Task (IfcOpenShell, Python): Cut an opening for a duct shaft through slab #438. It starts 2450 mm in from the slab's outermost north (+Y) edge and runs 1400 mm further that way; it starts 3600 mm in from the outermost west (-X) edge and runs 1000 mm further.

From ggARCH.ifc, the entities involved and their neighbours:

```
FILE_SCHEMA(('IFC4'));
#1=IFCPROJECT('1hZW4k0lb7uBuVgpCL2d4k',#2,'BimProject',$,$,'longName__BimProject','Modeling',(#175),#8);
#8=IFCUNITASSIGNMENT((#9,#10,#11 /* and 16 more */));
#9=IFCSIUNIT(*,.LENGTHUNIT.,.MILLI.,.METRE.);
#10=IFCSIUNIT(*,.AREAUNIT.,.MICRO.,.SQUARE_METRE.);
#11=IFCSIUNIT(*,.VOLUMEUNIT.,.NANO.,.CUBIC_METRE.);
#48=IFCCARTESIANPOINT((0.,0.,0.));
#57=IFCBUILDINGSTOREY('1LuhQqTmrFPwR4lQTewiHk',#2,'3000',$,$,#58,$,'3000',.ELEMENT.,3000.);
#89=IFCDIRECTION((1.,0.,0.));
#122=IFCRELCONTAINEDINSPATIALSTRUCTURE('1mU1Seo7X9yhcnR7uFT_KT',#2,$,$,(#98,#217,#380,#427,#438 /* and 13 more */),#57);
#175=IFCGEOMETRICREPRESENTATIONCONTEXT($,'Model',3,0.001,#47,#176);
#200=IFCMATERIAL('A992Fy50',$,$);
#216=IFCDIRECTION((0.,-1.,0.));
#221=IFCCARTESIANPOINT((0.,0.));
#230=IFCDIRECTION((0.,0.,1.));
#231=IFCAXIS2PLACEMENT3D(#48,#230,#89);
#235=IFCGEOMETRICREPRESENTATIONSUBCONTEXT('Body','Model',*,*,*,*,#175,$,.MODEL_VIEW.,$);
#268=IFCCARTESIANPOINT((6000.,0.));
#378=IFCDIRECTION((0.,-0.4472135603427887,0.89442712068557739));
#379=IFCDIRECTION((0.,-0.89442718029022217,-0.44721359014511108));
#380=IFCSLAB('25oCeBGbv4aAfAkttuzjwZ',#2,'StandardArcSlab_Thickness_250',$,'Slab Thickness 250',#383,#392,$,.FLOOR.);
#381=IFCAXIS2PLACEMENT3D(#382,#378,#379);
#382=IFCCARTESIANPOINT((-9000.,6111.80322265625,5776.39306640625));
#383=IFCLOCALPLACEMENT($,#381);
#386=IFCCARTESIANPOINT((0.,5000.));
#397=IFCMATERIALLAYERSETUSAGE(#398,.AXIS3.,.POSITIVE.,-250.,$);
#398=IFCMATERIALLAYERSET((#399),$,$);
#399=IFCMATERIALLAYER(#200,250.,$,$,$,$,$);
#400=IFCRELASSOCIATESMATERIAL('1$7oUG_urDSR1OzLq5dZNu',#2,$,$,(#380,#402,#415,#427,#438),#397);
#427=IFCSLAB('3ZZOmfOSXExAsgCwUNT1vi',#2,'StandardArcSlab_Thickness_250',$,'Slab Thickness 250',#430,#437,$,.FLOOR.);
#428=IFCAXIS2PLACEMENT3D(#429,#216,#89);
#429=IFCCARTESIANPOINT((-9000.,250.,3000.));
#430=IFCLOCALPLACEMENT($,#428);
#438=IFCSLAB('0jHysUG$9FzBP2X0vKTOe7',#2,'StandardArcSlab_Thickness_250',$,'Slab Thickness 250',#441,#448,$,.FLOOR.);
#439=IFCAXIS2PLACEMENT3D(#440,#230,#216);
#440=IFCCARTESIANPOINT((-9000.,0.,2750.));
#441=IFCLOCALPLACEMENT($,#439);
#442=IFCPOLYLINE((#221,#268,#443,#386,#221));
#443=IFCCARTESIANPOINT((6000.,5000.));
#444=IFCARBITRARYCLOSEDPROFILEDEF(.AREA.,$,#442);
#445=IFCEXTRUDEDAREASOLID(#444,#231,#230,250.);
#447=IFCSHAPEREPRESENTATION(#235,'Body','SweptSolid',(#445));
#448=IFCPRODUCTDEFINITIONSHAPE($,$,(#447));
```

```python
import numpy as np
import ifcopenshell
import ifcopenshell.api.feature
import ifcopenshell.api.geometry
import ifcopenshell.api.root
import ifcopenshell.geom
import ifcopenshell.util.placement
import ifcopenshell.util.representation
import ifcopenshell.util.shape
import ifcopenshell.util.unit

model = ifcopenshell.open("ggARCH.ifc")
unit_scale = ifcopenshell.util.unit.calculate_unit_scale(model)
settings = ifcopenshell.geom.settings()


def volume(element):
    """Net volume in cubic metres, openings subtracted."""
    shape = ifcopenshell.geom.create_shape(settings, element)
    return ifcopenshell.util.shape.get_volume(shape.geometry)


slab = model.by_guid("0jHysUG$9FzBP2X0vKTOe7")
before = volume(slab)

# Extent in the slab's own axes, in metres. The edges named are its -X and -Y sides.
slab_shape = ifcopenshell.geom.create_shape(settings, slab)
vertices = ifcopenshell.util.shape.get_vertices(slab_shape.geometry)
x_min, y_min, bottom = vertices.min(axis=0)
top = vertices[:, 2].max()

opening = ifcopenshell.api.root.create_entity(model, ifc_class="IfcOpeningElement", name="Duct shaft opening", predefined_type="OPENING")
context = ifcopenshell.util.representation.get_context(model, "Model", "Body", "MODEL_VIEW")
width, depth = 1.4, 1
outline = [(0.0, 0.0), (width, 0.0), (width, depth), (0.0, depth), (0.0, 0.0)]
# Overshoot both faces by 50 mm so the cut is clean.
shape = ifcopenshell.api.geometry.add_slab_representation(
    model, context=context, depth=top - bottom + 0.1, polyline=outline
)
ifcopenshell.api.geometry.assign_representation(model, product=opening, representation=shape)

matrix = ifcopenshell.util.placement.get_local_placement(slab.ObjectPlacement)
matrix[:, 3] = matrix @ np.append(np.array([x_min + 2.45, y_min + 3.6, bottom - 0.05]) / unit_scale, 1.0)
ifcopenshell.api.geometry.edit_object_placement(model, product=opening, matrix=matrix, is_si=False)
ifcopenshell.api.feature.add_feature(model, feature=opening, element=slab)

after = volume(slab)

print(f"slab volume {before:.3f} -> {after:.3f} m3")

model.write("ggARCH_v2.ifc")
```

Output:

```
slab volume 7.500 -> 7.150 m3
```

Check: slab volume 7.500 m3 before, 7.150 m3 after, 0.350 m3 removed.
